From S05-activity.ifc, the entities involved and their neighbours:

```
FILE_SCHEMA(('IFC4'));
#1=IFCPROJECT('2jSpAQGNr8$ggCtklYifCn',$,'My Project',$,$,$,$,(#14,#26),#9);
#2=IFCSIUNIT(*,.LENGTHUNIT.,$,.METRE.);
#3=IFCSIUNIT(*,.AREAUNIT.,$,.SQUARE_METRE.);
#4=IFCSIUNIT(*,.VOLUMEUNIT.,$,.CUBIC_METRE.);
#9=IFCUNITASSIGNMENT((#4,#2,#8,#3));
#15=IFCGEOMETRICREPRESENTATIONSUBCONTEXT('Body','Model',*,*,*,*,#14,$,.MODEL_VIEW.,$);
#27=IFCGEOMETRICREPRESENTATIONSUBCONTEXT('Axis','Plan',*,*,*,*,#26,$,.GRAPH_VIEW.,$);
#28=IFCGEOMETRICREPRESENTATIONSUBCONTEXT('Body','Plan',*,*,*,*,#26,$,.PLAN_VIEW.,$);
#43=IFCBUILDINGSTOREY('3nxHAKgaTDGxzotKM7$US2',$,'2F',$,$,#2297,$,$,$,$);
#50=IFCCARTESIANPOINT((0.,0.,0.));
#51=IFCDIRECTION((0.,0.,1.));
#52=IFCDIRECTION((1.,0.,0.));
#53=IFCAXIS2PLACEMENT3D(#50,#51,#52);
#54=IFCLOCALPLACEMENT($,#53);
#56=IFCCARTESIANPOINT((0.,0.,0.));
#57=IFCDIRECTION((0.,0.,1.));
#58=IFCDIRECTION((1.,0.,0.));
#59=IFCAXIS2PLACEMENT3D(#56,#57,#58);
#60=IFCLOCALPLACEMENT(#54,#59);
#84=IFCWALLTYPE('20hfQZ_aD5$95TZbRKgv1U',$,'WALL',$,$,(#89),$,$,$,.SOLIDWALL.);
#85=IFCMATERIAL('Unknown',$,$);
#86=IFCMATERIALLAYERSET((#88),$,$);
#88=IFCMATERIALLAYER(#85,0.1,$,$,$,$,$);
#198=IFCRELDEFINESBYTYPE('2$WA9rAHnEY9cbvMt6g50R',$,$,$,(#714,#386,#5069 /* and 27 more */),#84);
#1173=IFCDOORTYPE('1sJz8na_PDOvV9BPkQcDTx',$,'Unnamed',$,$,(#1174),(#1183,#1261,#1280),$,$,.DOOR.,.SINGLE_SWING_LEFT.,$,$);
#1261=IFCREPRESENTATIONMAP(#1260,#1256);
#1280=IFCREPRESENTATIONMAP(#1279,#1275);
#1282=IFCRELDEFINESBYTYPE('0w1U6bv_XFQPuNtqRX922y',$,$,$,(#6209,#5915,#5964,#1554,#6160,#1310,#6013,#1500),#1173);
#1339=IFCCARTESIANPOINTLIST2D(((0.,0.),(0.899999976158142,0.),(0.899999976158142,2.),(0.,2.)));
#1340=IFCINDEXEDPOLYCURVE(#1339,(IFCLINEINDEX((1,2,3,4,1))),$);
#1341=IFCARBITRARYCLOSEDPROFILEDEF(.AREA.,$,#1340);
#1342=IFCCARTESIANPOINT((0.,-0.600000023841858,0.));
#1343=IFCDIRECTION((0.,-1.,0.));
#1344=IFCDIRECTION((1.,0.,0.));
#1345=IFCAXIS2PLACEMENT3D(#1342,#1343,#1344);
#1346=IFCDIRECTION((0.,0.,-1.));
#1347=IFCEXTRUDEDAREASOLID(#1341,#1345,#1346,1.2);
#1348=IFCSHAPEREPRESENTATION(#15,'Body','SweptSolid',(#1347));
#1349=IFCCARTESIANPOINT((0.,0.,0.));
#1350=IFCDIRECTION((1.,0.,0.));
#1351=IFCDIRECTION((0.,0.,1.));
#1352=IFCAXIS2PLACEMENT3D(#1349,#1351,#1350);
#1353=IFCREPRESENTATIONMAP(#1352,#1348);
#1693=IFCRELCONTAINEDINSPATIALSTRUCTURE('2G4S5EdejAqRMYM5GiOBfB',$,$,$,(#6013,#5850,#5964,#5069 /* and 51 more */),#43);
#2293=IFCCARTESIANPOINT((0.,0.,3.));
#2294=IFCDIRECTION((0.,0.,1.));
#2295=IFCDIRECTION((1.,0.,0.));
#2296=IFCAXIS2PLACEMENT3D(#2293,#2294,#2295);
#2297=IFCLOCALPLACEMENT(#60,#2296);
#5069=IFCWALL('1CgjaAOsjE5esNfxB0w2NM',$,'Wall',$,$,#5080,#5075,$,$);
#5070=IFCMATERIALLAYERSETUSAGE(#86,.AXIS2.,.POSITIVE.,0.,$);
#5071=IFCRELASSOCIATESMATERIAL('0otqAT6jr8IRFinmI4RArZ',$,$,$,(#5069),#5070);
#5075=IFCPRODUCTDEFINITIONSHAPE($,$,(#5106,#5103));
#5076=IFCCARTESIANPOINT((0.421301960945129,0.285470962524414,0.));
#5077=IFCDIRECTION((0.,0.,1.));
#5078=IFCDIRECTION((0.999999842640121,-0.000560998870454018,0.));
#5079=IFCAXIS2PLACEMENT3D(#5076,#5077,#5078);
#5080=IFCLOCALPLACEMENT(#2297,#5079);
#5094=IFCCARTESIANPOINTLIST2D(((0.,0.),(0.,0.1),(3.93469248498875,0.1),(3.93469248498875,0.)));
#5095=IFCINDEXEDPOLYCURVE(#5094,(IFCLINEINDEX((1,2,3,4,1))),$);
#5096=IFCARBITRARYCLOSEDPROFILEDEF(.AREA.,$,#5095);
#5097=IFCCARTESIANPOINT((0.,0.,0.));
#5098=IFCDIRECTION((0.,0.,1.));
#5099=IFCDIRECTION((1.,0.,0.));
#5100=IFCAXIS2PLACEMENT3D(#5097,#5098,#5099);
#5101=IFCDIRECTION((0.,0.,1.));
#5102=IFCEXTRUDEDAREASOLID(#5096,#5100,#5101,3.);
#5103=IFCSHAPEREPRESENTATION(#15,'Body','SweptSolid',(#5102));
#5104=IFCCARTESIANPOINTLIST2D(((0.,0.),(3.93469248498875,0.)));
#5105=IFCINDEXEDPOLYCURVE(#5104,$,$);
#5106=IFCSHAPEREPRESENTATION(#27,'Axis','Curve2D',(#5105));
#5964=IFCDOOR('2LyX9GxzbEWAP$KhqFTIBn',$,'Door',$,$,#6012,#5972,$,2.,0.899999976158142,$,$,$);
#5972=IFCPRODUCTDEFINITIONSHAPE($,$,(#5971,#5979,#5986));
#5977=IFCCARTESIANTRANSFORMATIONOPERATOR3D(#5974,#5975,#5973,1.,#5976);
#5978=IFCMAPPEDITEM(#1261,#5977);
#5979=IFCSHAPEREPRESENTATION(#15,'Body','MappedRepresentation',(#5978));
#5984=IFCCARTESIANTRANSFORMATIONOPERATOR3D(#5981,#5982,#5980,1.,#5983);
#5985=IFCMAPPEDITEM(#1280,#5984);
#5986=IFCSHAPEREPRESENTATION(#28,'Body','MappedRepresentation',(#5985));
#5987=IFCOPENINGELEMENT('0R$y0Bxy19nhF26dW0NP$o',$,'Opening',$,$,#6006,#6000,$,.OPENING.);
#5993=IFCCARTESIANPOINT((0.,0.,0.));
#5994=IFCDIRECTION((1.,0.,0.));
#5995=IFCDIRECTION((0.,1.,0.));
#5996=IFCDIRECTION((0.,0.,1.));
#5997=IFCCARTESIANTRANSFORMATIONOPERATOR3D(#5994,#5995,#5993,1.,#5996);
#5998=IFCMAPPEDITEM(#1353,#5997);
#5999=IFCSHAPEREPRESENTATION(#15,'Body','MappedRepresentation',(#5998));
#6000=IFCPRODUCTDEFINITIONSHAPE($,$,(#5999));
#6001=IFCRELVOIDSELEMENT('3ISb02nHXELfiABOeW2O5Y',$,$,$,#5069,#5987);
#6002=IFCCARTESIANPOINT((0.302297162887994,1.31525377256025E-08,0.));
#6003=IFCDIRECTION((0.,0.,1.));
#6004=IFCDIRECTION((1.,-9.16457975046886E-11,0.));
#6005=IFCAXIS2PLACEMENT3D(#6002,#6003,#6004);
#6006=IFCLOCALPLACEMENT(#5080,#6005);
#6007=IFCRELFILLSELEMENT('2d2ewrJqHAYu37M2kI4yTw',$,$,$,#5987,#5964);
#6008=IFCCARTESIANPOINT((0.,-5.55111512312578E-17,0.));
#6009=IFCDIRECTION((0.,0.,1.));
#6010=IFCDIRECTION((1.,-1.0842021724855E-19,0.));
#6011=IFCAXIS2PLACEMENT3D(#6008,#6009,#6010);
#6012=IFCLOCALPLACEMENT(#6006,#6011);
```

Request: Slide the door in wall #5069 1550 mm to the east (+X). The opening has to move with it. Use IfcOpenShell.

```python
import ifcopenshell
import ifcopenshell.api.geometry
import ifcopenshell.util.placement
import ifcopenshell.util.unit

model = ifcopenshell.open("S05-activity.ifc")
unit_scale = ifcopenshell.util.unit.calculate_unit_scale(model)

door = model.by_guid("2LyX9GxzbEWAP$KhqFTIBn")
opening = door.FillsVoids[0].RelatingOpeningElement
wall = opening.VoidsElements[0].RelatingBuildingElement

wall_matrix = ifcopenshell.util.placement.get_local_placement(wall.ObjectPlacement)
shift = wall_matrix[:3, 0] * 1.55 / unit_scale
before = ifcopenshell.util.placement.get_local_placement(door.ObjectPlacement)[:3, 3].copy()

# The door is placed relative to its opening, so it follows when the opening moves.
matrix = ifcopenshell.util.placement.get_local_placement(opening.ObjectPlacement)
matrix[:3, 3] += shift
ifcopenshell.api.geometry.edit_object_placement(
    model, product=opening, matrix=matrix, is_si=False, should_transform_children=True
)

after = ifcopenshell.util.placement.get_local_placement(door.ObjectPlacement)[:3, 3]
print("door moved by", (after - before).round(3) + 0.0)

model.write("S05-activity_rev.ifc")
```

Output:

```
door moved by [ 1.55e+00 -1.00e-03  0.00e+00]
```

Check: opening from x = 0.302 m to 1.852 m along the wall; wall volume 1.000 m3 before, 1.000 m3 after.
